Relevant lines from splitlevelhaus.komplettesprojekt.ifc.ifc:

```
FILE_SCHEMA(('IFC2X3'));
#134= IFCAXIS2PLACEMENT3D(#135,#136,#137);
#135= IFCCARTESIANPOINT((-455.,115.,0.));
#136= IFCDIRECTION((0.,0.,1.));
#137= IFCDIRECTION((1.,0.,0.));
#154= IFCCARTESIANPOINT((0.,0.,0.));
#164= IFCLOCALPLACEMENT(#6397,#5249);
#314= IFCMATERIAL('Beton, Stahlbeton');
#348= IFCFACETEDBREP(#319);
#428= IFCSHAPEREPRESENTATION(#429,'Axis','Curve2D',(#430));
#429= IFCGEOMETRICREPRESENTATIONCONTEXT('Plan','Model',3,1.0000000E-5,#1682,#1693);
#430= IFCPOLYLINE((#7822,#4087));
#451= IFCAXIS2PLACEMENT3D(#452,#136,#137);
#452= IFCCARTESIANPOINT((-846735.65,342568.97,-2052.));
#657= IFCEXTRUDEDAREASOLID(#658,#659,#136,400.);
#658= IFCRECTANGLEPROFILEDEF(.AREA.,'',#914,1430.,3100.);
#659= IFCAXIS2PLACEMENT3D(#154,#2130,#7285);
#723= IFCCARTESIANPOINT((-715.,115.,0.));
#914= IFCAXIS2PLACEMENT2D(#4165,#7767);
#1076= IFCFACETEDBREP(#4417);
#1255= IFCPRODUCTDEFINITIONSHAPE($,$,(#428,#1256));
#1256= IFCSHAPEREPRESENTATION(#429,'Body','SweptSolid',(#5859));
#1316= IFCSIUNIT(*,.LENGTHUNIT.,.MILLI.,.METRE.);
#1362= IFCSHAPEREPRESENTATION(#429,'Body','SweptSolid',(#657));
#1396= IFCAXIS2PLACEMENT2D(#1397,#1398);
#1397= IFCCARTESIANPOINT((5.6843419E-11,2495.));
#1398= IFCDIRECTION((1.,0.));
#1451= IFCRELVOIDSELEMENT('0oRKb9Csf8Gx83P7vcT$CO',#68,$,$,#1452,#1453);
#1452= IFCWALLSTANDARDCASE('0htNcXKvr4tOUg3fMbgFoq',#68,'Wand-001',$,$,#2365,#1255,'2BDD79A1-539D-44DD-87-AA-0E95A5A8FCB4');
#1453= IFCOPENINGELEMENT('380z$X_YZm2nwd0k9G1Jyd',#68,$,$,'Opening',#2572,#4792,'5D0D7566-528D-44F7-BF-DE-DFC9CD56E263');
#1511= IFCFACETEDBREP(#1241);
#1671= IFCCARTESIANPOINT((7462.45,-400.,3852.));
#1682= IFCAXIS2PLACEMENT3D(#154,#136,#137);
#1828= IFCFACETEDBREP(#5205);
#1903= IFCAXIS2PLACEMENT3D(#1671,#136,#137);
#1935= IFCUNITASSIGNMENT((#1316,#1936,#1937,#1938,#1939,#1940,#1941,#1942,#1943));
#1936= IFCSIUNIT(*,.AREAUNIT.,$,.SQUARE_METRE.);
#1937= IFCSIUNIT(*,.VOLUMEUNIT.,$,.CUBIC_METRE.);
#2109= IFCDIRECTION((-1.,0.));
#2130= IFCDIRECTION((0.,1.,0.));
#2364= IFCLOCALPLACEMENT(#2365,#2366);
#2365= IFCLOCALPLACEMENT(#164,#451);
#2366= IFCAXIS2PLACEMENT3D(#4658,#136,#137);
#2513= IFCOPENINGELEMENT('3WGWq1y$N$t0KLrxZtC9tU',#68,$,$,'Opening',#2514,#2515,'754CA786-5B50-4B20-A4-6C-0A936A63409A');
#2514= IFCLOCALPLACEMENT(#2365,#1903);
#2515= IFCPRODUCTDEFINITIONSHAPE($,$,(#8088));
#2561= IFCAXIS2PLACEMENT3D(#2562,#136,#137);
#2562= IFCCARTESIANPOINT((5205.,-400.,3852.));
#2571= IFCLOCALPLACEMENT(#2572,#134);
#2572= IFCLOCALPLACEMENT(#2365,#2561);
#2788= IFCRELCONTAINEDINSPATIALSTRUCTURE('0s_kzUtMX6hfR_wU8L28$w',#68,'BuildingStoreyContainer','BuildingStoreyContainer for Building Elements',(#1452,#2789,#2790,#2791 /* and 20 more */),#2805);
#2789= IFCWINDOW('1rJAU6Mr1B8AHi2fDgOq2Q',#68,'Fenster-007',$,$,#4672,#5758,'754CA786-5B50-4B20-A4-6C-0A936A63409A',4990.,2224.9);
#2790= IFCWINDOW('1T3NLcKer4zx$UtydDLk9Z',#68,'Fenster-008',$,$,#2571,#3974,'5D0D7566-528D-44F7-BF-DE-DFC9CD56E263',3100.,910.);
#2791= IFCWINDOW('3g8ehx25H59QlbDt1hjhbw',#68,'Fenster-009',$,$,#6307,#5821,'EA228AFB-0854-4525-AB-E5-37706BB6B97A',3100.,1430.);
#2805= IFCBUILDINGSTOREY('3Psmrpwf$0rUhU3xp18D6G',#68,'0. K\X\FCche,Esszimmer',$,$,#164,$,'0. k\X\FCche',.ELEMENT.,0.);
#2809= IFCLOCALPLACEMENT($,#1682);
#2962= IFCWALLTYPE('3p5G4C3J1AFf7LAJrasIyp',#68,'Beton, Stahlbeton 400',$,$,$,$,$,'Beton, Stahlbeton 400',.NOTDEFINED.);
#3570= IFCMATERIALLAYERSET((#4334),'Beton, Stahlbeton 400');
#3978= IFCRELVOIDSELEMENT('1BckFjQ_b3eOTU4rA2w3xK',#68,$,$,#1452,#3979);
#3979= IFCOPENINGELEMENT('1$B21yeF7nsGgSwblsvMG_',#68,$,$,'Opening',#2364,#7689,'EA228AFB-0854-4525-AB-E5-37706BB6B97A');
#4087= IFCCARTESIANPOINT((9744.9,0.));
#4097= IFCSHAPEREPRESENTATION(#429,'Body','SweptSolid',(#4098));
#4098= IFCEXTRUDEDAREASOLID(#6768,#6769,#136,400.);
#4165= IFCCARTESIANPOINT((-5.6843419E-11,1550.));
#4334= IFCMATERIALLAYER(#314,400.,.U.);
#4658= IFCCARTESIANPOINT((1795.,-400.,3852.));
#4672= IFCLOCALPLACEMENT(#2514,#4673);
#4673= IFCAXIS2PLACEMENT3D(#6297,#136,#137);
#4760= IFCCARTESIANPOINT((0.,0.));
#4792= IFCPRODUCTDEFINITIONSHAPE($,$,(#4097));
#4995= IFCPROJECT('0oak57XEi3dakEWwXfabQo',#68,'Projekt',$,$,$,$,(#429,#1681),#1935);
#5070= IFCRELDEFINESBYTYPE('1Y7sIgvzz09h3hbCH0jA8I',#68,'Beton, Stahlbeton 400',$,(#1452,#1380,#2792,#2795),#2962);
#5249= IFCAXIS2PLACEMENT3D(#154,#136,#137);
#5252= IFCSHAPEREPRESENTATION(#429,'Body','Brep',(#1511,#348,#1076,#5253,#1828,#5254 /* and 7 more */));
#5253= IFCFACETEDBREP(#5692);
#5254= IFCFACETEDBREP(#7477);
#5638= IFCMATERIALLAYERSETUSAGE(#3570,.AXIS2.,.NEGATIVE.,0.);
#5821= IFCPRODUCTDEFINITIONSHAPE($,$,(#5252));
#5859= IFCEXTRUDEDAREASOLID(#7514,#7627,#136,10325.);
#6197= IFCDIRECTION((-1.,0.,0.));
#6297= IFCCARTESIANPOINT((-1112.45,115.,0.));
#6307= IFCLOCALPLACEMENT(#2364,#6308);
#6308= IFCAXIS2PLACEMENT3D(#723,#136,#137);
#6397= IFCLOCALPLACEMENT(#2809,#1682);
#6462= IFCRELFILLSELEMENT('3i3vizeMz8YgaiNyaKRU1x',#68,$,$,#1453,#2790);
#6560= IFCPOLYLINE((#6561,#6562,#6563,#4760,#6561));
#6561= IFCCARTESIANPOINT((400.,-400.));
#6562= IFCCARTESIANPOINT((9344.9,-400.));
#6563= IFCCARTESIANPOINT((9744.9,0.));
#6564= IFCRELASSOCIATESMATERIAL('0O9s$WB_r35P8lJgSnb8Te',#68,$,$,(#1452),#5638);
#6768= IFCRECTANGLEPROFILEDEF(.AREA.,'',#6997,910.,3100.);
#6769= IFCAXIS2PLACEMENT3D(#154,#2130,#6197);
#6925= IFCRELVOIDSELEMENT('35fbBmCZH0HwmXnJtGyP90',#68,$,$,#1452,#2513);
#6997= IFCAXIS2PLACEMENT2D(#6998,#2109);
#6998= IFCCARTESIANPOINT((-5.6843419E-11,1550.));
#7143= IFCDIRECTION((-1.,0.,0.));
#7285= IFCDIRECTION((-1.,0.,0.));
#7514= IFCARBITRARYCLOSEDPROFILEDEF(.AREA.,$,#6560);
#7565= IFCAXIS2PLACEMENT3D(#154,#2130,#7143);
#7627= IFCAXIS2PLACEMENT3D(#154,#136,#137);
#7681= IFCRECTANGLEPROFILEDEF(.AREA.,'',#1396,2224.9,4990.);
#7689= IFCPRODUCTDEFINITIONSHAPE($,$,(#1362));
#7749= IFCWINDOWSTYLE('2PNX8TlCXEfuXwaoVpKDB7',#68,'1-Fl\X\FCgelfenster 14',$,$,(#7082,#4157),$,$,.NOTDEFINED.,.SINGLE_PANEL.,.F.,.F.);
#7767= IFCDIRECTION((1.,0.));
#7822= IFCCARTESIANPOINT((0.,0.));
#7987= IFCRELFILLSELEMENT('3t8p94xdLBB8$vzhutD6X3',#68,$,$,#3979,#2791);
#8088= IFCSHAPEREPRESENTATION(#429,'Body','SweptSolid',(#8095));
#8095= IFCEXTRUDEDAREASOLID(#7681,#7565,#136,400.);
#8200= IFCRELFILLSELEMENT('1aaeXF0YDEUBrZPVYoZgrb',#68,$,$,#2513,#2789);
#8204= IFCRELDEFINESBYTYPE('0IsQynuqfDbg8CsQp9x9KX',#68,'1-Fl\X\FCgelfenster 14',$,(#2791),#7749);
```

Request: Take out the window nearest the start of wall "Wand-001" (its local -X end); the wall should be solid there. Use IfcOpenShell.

```python
import ifcopenshell
import ifcopenshell.api.feature
import ifcopenshell.api.root
import ifcopenshell.geom
import ifcopenshell.util.shape

model = ifcopenshell.open("splitlevelhaus.komplettesprojekt.ifc.ifc")
settings = ifcopenshell.geom.settings()


def volume(element):
    """Net volume in cubic metres, openings subtracted."""
    shape = ifcopenshell.geom.create_shape(settings, element)
    return ifcopenshell.util.shape.get_volume(shape.geometry)


window = model.by_guid("3g8ehx25H59QlbDt1hjhbw")
opening = window.FillsVoids[0].RelatingOpeningElement
wall = opening.VoidsElements[0].RelatingBuildingElement
before = volume(wall)

ifcopenshell.api.root.remove_product(model, product=window)
ifcopenshell.api.feature.remove_feature(model, feature=opening)

after = volume(wall)

print(f"wall volume {before:.3f} -> {after:.3f} m3")

model.write("splitlevelhaus.komplettesprojekt.ifc_rev.ifc")
```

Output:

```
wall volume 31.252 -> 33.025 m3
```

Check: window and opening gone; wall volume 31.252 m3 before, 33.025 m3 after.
